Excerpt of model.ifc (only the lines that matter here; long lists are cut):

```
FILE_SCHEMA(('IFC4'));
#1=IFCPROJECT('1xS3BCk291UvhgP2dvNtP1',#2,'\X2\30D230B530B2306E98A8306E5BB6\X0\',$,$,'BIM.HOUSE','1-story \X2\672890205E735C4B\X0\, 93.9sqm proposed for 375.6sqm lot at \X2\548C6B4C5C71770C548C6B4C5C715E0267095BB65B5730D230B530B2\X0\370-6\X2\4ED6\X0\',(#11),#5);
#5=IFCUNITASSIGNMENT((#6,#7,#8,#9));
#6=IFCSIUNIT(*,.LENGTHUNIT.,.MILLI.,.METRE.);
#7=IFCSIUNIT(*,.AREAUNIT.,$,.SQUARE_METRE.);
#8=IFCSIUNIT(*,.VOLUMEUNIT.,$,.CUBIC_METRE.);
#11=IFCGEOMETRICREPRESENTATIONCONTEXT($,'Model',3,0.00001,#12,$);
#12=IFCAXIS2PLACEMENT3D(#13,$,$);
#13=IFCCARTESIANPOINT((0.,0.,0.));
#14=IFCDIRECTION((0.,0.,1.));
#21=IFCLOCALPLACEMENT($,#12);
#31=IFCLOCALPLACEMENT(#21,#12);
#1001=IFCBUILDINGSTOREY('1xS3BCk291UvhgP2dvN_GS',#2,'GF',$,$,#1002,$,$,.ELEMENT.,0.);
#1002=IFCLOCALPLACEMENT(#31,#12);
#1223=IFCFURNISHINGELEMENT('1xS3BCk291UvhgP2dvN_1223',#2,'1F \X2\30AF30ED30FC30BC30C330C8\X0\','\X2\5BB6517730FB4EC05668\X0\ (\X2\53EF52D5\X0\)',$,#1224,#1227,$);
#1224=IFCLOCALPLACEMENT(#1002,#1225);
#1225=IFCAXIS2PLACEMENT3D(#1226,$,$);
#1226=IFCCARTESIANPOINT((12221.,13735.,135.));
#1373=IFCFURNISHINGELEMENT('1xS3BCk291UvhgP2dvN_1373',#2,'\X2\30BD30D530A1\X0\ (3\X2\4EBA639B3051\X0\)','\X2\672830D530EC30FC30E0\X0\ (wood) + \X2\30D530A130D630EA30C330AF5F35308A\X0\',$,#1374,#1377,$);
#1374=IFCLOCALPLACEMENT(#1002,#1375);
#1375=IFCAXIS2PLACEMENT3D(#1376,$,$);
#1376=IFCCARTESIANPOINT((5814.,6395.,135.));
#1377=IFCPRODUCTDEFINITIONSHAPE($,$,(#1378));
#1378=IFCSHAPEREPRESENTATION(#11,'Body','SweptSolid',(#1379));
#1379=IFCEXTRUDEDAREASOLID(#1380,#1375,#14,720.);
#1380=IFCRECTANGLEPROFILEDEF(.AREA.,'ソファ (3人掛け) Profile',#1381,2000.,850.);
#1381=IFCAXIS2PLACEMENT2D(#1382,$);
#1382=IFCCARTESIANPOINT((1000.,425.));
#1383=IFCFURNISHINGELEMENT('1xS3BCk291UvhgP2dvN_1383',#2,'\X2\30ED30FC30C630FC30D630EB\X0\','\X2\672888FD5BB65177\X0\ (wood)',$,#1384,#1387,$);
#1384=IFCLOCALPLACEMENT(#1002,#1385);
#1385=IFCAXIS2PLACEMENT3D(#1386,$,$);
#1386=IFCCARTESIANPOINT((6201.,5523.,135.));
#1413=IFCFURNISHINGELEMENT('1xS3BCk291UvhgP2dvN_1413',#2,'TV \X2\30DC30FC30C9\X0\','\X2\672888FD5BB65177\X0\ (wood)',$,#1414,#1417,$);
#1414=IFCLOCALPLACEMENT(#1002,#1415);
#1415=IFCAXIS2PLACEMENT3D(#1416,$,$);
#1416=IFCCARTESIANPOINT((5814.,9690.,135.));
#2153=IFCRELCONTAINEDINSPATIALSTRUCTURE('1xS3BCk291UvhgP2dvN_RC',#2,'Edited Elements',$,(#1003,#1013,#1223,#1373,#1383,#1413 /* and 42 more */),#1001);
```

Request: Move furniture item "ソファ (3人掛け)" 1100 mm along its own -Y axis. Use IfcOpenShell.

```python
import ifcopenshell
import ifcopenshell.api.geometry
import ifcopenshell.util.placement
import ifcopenshell.util.unit

model = ifcopenshell.open("model.ifc")
unit_scale = ifcopenshell.util.unit.calculate_unit_scale(model)

item = model.by_guid("1xS3BCk291UvhgP2dvN_1373")
matrix = ifcopenshell.util.placement.get_local_placement(item.ObjectPlacement)
matrix[:3, 3] -= matrix[:3, 1] * 1.1 / unit_scale
ifcopenshell.api.geometry.edit_object_placement(model, product=item, matrix=matrix, is_si=False)

print(ifcopenshell.util.placement.get_local_placement(item.ObjectPlacement).round(3) + 0.0)

model.write("model_rev.ifc")
```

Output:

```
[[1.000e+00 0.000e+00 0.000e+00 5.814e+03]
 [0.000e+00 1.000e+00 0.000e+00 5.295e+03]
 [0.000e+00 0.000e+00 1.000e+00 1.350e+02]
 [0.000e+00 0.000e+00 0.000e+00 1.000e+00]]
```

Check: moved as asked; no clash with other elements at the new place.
